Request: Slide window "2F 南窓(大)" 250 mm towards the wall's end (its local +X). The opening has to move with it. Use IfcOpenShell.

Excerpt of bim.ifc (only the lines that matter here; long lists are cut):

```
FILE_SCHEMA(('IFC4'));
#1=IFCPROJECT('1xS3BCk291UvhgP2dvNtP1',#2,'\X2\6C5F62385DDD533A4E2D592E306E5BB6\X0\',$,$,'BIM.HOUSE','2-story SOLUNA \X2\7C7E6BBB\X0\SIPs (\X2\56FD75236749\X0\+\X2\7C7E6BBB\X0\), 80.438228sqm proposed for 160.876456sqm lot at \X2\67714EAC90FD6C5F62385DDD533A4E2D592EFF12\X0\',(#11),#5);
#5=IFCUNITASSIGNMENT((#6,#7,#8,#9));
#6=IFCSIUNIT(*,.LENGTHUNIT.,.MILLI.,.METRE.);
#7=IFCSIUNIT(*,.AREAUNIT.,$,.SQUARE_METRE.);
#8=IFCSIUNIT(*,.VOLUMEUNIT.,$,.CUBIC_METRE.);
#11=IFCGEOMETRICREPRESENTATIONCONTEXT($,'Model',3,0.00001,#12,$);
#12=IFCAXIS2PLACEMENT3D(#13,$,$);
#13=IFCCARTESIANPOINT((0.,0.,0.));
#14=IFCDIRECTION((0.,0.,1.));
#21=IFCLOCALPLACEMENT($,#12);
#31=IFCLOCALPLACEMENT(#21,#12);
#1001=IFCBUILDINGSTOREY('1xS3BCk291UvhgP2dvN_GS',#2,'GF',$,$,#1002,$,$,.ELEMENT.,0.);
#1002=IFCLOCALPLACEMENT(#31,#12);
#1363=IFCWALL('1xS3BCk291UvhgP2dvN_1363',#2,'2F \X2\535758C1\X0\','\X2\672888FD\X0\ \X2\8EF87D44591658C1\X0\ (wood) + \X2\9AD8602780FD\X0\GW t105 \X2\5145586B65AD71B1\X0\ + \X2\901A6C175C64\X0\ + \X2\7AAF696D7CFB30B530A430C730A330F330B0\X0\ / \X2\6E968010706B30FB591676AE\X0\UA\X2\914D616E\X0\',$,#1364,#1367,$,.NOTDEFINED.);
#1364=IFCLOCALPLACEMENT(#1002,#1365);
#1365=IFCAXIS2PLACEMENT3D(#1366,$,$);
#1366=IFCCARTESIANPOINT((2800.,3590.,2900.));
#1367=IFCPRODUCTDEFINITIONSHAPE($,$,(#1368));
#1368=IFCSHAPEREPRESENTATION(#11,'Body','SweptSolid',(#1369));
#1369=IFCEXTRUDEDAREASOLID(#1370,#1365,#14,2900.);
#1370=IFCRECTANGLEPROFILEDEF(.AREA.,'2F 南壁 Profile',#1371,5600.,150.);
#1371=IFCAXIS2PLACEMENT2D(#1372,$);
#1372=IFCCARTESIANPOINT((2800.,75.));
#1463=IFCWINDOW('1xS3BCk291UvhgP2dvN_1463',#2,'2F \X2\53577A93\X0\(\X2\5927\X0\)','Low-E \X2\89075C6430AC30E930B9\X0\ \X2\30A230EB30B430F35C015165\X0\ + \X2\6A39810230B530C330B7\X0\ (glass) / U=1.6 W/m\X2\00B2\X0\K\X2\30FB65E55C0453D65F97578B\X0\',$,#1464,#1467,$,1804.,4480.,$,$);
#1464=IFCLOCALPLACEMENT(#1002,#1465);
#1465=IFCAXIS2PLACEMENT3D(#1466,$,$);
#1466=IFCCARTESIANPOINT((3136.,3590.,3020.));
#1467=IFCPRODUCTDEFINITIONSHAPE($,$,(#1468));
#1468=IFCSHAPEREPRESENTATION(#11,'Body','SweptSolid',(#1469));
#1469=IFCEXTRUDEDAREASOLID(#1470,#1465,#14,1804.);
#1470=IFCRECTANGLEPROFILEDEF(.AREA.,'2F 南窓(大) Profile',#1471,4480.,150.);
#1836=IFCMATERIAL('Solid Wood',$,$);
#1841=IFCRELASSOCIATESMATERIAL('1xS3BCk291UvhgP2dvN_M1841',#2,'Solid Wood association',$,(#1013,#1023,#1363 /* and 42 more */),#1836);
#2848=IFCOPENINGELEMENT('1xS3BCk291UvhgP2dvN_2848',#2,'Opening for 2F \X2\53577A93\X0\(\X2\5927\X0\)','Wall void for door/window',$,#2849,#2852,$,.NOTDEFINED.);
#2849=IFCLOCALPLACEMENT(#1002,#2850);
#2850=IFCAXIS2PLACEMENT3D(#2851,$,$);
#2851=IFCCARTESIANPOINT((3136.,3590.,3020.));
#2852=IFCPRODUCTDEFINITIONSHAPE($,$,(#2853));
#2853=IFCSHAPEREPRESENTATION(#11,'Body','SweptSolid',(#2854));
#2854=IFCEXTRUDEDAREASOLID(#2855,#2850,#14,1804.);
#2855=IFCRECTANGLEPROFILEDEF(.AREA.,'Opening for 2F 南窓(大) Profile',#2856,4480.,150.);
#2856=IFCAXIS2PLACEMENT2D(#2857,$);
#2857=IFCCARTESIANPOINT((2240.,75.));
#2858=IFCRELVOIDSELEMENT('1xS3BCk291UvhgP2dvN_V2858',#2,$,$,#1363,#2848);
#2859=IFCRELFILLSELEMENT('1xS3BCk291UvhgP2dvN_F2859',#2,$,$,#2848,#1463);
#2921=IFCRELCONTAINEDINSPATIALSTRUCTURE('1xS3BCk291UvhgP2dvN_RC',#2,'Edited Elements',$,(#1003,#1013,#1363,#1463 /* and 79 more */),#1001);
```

```python
import ifcopenshell
import ifcopenshell.api.geometry
import ifcopenshell.util.placement
import ifcopenshell.util.unit

model = ifcopenshell.open("bim.ifc")
unit_scale = ifcopenshell.util.unit.calculate_unit_scale(model)

window = model.by_id(1463)
opening = window.FillsVoids[0].RelatingOpeningElement
wall = opening.VoidsElements[0].RelatingBuildingElement

wall_matrix = ifcopenshell.util.placement.get_local_placement(wall.ObjectPlacement)
shift = wall_matrix[:3, 0] * 0.25 / unit_scale
before = ifcopenshell.util.placement.get_local_placement(window.ObjectPlacement)[:3, 3].copy()

# The window is not placed relative to its opening, so move both.
for product in (opening, window):
    matrix = ifcopenshell.util.placement.get_local_placement(product.ObjectPlacement)
    matrix[:3, 3] += shift
    ifcopenshell.api.geometry.edit_object_placement(model, product=product, matrix=matrix, is_si=False)

after = ifcopenshell.util.placement.get_local_placement(window.ObjectPlacement)[:3, 3]
print("window moved by", (after - before).round(3) + 0.0)

model.write("bim_rev.ifc")
```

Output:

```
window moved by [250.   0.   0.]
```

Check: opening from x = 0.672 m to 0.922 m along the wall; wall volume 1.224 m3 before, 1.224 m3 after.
